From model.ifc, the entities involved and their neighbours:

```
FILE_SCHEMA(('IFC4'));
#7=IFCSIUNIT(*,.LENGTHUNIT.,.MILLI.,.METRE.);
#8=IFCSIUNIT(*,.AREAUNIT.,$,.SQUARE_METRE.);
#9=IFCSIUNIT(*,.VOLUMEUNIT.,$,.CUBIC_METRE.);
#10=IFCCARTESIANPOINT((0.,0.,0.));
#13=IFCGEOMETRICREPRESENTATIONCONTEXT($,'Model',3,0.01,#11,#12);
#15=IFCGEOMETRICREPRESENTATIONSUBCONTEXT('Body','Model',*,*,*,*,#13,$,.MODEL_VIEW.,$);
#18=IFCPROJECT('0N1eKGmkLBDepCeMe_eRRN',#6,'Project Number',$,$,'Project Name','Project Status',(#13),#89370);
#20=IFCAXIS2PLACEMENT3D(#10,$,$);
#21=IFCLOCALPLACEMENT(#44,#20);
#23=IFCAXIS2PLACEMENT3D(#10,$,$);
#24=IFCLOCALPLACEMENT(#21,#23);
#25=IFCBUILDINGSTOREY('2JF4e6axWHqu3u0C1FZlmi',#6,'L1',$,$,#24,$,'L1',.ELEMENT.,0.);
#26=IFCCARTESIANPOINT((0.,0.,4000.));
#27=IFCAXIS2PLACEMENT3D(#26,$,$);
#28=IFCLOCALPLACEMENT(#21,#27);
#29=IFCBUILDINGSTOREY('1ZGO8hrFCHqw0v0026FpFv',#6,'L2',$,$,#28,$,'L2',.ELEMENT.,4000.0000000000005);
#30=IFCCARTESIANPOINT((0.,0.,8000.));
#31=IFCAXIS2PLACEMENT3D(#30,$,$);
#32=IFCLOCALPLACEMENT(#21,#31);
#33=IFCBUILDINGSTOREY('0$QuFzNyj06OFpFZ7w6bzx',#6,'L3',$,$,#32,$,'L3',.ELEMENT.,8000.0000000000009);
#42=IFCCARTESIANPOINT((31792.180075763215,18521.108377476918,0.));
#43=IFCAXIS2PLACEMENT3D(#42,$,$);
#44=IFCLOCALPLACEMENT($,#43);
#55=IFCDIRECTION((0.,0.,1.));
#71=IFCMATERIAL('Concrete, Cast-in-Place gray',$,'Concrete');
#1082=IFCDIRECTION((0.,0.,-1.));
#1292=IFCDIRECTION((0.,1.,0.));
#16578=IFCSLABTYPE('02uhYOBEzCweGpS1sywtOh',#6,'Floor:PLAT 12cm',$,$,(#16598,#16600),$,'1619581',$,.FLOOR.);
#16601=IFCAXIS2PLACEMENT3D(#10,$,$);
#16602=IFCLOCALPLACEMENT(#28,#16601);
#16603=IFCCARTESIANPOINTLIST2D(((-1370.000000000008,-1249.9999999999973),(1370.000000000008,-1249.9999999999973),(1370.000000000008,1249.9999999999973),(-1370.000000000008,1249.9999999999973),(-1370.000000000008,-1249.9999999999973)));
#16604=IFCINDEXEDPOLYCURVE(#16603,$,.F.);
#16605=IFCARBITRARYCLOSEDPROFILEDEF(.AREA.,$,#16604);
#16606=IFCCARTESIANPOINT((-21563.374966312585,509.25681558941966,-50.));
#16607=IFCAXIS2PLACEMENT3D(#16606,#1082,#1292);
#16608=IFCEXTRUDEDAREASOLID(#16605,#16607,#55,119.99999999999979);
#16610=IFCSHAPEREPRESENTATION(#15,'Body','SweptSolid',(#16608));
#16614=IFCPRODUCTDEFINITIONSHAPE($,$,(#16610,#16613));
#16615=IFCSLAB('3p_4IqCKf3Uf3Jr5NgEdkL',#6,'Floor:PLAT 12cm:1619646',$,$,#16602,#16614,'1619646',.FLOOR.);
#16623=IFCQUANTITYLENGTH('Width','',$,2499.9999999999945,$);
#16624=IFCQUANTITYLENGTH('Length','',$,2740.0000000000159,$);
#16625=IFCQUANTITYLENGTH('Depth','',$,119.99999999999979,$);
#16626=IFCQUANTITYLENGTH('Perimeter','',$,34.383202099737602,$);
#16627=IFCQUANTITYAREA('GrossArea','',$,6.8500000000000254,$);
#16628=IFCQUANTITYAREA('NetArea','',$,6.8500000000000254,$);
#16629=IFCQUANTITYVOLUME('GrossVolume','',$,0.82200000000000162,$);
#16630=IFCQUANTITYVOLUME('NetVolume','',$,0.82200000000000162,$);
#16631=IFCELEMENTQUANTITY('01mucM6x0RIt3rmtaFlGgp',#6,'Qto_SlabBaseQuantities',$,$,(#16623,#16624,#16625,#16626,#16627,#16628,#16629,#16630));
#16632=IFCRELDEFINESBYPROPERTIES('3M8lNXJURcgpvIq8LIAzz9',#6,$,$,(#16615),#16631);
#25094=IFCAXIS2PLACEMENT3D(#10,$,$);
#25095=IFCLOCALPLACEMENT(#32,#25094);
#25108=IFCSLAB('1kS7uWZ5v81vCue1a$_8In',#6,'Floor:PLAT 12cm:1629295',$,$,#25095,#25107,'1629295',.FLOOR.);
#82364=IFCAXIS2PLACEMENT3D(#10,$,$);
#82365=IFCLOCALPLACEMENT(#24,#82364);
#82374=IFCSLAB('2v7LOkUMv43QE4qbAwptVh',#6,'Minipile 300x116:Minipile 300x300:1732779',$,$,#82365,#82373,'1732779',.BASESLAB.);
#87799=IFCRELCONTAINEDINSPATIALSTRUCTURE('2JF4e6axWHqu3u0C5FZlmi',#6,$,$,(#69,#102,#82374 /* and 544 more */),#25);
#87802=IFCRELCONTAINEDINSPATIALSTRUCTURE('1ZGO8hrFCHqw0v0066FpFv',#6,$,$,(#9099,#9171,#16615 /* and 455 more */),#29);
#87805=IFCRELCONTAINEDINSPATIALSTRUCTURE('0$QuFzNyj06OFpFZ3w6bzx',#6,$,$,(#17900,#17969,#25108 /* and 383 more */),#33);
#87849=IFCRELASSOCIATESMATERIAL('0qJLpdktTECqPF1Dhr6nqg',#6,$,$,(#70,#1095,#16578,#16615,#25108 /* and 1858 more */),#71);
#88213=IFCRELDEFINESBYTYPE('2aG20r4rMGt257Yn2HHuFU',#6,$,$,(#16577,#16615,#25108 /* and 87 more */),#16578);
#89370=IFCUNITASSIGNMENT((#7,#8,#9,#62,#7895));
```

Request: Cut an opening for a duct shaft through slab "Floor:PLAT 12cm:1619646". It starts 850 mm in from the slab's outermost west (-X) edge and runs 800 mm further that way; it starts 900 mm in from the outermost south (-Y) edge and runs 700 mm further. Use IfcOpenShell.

```python
import numpy as np
import ifcopenshell
import ifcopenshell.api.feature
import ifcopenshell.api.geometry
import ifcopenshell.api.pset
import ifcopenshell.api.root
import ifcopenshell.geom
import ifcopenshell.util.element
import ifcopenshell.util.placement
import ifcopenshell.util.representation
import ifcopenshell.util.shape
import ifcopenshell.util.unit

model = ifcopenshell.open("model.ifc")
unit_scale = ifcopenshell.util.unit.calculate_unit_scale(model)
area_scale = ifcopenshell.util.unit.calculate_unit_scale(model, "AREAUNIT")
volume_scale = ifcopenshell.util.unit.calculate_unit_scale(model, "VOLUMEUNIT")
settings = ifcopenshell.geom.settings()


def volume(element):
    """Net volume in cubic metres, openings subtracted."""
    shape = ifcopenshell.geom.create_shape(settings, element)
    return ifcopenshell.util.shape.get_volume(shape.geometry)


slab = model.by_guid("3p_4IqCKf3Uf3Jr5NgEdkL")
before = volume(slab)

# Extent in the slab's own axes, in metres. The edges named are its -X and -Y sides.
slab_shape = ifcopenshell.geom.create_shape(settings, slab)
vertices = ifcopenshell.util.shape.get_vertices(slab_shape.geometry)
x_min, y_min, bottom = vertices.min(axis=0)
top = vertices[:, 2].max()

opening = ifcopenshell.api.root.create_entity(model, ifc_class="IfcOpeningElement", name="Duct shaft opening", predefined_type="OPENING")
context = ifcopenshell.util.representation.get_context(model, "Model", "Body", "MODEL_VIEW")
width, depth = 0.8, 0.7
outline = [(0.0, 0.0), (width, 0.0), (width, depth), (0.0, depth), (0.0, 0.0)]
# Overshoot both faces by 50 mm so the cut is clean.
shape = ifcopenshell.api.geometry.add_slab_representation(
    model, context=context, depth=top - bottom + 0.1, polyline=outline
)
ifcopenshell.api.geometry.assign_representation(model, product=opening, representation=shape)

matrix = ifcopenshell.util.placement.get_local_placement(slab.ObjectPlacement)
matrix[:, 3] = matrix @ np.append(np.array([x_min + 0.85, y_min + 0.9, bottom - 0.05]) / unit_scale, 1.0)
ifcopenshell.api.geometry.edit_object_placement(model, product=opening, matrix=matrix, is_si=False)
ifcopenshell.api.feature.add_feature(model, feature=opening, element=slab)

after = volume(slab)

# Update the slab's stored quantities.
qto = model.by_id(ifcopenshell.util.element.get_pset(slab, "Qto_SlabBaseQuantities", should_inherit=False)["id"])
ifcopenshell.api.pset.edit_qto(model, qto=qto, properties={
    "NetArea": after / (top - bottom) / area_scale,
    "NetVolume": after / volume_scale,
})

print(f"slab volume {before:.3f} -> {after:.3f} m3")

model.write("model_updated.ifc")
```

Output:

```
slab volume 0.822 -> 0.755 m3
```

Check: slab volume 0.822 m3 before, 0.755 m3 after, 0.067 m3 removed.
